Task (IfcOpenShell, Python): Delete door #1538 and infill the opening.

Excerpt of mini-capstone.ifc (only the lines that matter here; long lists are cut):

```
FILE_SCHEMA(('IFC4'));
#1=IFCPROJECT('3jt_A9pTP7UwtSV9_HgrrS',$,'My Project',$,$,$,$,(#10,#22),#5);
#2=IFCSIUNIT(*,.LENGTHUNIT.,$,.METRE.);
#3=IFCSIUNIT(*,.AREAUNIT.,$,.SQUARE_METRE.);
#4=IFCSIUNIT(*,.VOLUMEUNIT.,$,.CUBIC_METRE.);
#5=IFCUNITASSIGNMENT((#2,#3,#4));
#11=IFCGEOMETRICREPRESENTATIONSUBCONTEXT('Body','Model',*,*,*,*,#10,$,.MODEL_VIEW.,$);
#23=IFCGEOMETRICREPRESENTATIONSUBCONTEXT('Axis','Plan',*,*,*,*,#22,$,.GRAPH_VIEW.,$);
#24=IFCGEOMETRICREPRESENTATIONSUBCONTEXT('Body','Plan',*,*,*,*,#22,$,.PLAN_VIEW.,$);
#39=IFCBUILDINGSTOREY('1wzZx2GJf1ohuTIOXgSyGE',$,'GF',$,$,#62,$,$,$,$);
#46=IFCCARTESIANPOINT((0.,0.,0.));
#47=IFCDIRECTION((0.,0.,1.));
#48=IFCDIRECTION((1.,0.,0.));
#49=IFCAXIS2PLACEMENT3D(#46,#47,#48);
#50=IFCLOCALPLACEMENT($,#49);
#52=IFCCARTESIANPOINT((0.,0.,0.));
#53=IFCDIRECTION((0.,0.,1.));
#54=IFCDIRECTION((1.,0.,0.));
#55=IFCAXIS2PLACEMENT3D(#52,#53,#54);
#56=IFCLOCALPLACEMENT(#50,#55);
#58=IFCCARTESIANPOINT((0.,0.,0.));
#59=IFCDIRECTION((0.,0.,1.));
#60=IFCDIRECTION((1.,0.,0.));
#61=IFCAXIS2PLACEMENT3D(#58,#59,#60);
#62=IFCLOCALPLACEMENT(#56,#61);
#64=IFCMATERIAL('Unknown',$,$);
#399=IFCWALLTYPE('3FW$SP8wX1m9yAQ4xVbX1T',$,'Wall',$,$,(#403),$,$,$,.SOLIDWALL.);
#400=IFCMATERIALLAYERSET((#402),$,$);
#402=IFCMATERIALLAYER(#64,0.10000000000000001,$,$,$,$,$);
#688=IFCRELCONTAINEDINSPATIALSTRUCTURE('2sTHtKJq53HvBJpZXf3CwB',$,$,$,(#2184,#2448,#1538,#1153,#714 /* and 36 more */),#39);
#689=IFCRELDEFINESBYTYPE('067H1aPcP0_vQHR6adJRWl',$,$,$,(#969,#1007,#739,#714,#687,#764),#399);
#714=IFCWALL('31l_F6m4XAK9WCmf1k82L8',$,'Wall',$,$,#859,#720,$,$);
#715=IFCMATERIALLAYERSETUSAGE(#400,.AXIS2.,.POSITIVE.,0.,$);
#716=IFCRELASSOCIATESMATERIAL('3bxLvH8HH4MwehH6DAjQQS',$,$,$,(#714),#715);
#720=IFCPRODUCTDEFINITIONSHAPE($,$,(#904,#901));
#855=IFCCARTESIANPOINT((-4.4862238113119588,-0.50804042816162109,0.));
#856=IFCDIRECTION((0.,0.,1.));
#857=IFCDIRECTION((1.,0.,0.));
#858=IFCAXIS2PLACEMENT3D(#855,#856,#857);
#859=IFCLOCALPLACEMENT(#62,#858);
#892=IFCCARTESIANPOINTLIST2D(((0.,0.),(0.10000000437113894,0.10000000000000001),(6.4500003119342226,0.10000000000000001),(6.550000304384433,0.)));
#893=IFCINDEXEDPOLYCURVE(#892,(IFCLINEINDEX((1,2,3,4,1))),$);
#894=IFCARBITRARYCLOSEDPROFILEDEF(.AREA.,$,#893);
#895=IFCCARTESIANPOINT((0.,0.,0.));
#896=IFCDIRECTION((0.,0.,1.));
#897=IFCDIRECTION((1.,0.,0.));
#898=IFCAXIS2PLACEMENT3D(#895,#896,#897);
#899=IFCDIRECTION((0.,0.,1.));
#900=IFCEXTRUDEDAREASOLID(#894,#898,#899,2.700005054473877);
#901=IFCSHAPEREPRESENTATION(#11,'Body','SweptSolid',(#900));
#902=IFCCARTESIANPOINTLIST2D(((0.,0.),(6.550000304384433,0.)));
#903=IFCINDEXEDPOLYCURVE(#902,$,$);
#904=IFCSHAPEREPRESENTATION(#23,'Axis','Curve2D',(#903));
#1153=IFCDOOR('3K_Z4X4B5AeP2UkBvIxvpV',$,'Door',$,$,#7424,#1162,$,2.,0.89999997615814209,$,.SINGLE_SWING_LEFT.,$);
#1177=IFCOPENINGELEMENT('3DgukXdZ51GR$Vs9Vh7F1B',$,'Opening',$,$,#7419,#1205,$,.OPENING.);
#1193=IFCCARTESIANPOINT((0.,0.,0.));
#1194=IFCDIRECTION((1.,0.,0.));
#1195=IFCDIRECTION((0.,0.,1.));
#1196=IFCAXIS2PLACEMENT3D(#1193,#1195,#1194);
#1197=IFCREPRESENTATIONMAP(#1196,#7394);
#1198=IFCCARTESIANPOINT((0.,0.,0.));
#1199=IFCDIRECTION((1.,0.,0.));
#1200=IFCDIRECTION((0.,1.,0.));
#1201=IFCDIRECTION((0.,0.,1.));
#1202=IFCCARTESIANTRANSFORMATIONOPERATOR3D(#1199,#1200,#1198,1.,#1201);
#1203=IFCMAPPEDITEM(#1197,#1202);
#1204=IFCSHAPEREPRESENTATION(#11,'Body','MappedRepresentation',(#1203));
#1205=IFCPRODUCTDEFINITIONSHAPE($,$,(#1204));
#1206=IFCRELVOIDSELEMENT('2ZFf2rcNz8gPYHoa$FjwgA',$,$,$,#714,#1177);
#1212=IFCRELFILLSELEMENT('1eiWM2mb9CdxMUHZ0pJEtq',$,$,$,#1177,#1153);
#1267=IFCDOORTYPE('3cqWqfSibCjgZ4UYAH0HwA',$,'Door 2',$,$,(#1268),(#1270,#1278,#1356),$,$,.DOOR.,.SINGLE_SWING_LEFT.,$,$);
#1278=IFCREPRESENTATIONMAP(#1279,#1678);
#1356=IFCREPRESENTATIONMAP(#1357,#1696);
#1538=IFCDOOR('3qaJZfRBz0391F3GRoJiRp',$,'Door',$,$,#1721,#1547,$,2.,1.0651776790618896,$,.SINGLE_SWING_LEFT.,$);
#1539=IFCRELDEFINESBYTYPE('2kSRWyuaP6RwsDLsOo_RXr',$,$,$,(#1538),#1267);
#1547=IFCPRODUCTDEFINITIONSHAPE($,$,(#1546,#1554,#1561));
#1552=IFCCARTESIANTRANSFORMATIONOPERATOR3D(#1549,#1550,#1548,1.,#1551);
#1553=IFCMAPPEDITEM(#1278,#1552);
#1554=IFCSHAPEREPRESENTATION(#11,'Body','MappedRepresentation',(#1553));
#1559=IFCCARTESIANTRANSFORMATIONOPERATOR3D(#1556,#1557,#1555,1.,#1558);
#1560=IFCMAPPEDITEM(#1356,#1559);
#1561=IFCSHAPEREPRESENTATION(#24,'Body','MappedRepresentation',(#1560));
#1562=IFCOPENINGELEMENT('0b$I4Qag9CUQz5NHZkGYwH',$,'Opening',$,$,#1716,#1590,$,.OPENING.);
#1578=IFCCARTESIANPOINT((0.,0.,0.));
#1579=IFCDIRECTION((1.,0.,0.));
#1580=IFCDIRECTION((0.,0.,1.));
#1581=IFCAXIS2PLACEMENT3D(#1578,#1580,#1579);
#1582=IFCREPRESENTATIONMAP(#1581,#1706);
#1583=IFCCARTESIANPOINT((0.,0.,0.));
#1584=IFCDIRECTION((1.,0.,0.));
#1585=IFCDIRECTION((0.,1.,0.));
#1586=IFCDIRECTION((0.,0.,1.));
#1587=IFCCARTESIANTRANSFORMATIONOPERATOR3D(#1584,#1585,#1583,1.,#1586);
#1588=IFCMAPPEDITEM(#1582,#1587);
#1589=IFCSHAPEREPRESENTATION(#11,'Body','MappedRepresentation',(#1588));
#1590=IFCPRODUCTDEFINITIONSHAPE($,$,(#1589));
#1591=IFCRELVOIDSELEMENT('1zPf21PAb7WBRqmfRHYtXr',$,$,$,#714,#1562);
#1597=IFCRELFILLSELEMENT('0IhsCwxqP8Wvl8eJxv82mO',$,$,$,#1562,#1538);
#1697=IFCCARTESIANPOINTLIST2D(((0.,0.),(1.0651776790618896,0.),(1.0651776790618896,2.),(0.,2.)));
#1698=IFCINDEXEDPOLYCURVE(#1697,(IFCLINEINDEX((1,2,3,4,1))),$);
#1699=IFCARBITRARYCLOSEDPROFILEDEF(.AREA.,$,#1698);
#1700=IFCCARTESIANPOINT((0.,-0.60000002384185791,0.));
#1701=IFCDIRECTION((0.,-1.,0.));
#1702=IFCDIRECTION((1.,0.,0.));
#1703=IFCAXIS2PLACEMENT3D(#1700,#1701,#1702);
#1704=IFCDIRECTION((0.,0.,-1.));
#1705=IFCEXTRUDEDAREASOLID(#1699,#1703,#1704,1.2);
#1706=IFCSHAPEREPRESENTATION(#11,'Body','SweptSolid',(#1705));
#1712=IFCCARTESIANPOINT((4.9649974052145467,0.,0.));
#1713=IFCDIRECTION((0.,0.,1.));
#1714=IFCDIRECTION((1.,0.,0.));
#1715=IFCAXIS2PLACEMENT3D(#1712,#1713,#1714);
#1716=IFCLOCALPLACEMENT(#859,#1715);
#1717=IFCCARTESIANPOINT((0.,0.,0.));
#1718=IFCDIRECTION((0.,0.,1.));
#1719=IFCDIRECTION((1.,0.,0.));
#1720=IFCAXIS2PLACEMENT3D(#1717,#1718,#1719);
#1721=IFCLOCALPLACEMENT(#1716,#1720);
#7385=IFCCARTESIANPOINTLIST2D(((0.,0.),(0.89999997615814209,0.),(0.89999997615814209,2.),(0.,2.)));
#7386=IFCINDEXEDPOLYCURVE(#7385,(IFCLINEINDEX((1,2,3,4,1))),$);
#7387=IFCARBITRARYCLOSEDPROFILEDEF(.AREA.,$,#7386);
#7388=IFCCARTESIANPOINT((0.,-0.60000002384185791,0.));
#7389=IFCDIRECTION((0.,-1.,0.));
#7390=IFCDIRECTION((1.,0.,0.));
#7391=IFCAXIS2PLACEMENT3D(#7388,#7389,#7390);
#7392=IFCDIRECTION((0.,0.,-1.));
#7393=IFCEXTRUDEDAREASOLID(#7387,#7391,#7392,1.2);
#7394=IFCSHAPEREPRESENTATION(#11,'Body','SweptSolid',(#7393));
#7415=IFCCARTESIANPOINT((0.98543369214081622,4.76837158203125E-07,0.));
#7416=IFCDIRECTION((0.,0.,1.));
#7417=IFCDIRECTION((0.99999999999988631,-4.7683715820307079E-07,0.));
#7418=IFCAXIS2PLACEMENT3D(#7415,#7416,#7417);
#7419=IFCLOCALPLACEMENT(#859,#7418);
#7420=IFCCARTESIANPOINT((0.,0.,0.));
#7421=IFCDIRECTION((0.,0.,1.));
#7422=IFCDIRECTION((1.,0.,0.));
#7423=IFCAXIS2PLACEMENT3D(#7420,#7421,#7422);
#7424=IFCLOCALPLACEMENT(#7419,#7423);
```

```python
import ifcopenshell
import ifcopenshell.api.feature
import ifcopenshell.api.root
import ifcopenshell.geom
import ifcopenshell.util.shape

model = ifcopenshell.open("mini-capstone.ifc")
settings = ifcopenshell.geom.settings()


def volume(element):
    """Net volume in cubic metres, openings subtracted."""
    shape = ifcopenshell.geom.create_shape(settings, element)
    return ifcopenshell.util.shape.get_volume(shape.geometry)


door = model.by_id(1538)
opening = door.FillsVoids[0].RelatingOpeningElement
wall = opening.VoidsElements[0].RelatingBuildingElement
before = volume(wall)

ifcopenshell.api.root.remove_product(model, product=door)
ifcopenshell.api.feature.remove_feature(model, feature=opening)

after = volume(wall)

print(f"wall volume {before:.3f} -> {after:.3f} m3")

model.write("mini-capstone-out.ifc")
```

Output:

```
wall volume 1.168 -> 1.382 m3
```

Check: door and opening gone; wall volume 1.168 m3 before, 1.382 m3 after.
